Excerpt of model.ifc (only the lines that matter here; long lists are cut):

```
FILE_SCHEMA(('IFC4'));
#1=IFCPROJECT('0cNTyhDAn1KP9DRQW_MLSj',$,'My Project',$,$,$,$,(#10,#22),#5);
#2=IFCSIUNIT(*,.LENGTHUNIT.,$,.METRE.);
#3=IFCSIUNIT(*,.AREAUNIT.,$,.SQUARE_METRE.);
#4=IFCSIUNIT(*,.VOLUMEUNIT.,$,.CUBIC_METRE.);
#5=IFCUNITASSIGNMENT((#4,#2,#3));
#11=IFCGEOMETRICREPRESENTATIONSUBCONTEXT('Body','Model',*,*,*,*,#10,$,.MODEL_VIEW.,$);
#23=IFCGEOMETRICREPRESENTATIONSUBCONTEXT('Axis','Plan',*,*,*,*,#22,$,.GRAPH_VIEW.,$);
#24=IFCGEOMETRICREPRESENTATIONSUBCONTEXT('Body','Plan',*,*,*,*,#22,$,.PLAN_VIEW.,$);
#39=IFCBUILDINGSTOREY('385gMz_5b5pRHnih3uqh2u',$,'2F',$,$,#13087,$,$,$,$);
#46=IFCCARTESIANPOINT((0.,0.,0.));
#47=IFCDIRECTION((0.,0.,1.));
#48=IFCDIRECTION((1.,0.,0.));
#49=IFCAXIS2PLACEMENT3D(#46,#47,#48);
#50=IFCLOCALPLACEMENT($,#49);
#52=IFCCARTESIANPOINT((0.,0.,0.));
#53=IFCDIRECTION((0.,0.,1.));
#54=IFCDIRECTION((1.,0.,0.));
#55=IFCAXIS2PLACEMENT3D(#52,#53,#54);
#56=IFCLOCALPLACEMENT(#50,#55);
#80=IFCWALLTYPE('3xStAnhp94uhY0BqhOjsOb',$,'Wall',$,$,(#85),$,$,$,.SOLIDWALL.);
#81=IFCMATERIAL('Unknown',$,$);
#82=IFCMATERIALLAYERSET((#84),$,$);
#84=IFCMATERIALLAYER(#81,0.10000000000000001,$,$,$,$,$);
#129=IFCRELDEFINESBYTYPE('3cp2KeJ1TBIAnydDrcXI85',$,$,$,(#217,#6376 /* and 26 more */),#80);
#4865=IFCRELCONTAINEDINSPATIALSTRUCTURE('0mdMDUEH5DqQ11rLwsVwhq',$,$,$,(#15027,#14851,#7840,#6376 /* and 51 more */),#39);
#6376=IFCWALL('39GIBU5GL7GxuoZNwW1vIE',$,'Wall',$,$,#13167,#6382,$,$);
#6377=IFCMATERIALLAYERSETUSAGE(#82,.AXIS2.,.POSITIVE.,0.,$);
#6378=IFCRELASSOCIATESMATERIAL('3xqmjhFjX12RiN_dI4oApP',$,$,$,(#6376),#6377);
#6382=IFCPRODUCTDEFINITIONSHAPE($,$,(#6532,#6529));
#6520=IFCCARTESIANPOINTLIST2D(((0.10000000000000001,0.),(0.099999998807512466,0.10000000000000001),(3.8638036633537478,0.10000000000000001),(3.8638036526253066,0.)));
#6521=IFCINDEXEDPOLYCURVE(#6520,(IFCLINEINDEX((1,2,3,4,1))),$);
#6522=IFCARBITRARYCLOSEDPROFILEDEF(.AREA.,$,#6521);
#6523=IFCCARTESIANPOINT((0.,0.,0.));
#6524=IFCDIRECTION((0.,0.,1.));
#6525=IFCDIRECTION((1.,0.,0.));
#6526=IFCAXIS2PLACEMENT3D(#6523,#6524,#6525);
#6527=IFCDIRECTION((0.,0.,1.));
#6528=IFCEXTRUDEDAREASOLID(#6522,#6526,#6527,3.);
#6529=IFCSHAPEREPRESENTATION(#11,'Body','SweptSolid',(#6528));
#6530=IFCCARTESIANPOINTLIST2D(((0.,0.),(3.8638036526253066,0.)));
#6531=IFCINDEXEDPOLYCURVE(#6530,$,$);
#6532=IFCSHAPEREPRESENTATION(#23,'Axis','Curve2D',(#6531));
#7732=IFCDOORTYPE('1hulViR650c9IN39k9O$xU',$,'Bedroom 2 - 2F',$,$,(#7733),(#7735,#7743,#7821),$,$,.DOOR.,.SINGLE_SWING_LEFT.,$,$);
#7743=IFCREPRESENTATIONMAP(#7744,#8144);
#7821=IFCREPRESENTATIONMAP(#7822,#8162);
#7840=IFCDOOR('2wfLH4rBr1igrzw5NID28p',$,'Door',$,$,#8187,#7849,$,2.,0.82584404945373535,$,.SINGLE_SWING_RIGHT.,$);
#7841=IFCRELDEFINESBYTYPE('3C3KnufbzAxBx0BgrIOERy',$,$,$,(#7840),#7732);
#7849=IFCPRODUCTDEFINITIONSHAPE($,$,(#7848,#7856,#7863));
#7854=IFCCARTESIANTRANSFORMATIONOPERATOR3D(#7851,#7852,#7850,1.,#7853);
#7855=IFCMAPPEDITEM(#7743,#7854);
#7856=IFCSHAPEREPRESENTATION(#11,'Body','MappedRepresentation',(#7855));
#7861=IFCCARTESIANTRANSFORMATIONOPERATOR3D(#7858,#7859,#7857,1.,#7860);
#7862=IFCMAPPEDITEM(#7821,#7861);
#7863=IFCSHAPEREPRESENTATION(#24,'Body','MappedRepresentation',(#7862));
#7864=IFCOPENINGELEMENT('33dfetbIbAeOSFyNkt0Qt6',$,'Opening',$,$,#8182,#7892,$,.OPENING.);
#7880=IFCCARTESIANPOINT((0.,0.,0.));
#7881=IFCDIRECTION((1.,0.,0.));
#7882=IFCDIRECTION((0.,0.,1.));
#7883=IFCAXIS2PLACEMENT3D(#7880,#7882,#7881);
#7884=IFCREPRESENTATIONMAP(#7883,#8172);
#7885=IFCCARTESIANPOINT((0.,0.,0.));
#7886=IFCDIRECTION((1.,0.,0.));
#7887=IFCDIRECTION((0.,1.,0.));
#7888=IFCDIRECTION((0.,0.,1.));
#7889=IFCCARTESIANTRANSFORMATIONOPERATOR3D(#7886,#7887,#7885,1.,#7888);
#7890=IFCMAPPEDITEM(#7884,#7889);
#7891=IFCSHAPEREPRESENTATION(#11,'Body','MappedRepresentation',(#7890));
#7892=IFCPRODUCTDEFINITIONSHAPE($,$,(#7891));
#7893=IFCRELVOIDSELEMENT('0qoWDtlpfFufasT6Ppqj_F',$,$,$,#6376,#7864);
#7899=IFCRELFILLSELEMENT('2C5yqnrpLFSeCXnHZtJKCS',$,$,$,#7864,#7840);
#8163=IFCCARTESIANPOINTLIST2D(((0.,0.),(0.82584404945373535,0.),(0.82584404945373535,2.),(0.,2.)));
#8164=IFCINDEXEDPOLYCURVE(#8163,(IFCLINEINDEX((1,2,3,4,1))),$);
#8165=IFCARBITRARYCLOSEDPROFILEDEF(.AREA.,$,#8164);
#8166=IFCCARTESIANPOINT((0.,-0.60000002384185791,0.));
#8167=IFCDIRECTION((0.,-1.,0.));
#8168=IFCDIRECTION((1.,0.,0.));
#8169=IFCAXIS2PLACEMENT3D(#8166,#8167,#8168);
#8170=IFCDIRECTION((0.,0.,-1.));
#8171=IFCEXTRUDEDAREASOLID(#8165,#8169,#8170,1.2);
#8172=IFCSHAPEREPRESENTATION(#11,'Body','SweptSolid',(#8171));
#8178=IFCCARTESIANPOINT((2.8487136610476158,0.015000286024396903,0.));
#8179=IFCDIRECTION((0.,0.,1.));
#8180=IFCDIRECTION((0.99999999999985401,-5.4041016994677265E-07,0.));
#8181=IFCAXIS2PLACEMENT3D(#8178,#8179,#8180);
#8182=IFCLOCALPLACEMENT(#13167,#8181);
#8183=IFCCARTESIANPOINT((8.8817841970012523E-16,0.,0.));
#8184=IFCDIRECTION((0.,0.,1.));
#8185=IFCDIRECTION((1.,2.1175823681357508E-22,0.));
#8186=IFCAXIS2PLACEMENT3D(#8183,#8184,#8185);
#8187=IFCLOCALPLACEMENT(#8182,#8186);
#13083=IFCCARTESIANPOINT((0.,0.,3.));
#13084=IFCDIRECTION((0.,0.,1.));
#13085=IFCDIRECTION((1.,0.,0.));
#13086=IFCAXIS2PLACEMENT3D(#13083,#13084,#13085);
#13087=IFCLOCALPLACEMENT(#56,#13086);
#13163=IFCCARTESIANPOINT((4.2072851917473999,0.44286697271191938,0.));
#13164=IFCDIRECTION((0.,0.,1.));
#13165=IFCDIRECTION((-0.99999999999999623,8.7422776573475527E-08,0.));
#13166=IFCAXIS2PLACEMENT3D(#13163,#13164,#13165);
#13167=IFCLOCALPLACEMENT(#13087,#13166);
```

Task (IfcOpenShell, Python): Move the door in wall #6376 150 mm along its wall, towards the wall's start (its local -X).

```python
import ifcopenshell
import ifcopenshell.api.geometry
import ifcopenshell.util.placement

model = ifcopenshell.open("model.ifc")

door = model.by_id(7840)
opening = door.FillsVoids[0].RelatingOpeningElement
wall = opening.VoidsElements[0].RelatingBuildingElement

wall_matrix = ifcopenshell.util.placement.get_local_placement(wall.ObjectPlacement)
shift = wall_matrix[:3, 0] * -0.15
before = ifcopenshell.util.placement.get_local_placement(door.ObjectPlacement)[:3, 3].copy()

# The door is placed relative to its opening, so it follows when the opening moves.
matrix = ifcopenshell.util.placement.get_local_placement(opening.ObjectPlacement)
matrix[:3, 3] += shift
ifcopenshell.api.geometry.edit_object_placement(
    model, product=opening, matrix=matrix, is_si=False, should_transform_children=True
)

after = ifcopenshell.util.placement.get_local_placement(door.ObjectPlacement)[:3, 3]
print("door moved by", (after - before).round(3) + 0.0)

model.write("model_updated.ifc")
```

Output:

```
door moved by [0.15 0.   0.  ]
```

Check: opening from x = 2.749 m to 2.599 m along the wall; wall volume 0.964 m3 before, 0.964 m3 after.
